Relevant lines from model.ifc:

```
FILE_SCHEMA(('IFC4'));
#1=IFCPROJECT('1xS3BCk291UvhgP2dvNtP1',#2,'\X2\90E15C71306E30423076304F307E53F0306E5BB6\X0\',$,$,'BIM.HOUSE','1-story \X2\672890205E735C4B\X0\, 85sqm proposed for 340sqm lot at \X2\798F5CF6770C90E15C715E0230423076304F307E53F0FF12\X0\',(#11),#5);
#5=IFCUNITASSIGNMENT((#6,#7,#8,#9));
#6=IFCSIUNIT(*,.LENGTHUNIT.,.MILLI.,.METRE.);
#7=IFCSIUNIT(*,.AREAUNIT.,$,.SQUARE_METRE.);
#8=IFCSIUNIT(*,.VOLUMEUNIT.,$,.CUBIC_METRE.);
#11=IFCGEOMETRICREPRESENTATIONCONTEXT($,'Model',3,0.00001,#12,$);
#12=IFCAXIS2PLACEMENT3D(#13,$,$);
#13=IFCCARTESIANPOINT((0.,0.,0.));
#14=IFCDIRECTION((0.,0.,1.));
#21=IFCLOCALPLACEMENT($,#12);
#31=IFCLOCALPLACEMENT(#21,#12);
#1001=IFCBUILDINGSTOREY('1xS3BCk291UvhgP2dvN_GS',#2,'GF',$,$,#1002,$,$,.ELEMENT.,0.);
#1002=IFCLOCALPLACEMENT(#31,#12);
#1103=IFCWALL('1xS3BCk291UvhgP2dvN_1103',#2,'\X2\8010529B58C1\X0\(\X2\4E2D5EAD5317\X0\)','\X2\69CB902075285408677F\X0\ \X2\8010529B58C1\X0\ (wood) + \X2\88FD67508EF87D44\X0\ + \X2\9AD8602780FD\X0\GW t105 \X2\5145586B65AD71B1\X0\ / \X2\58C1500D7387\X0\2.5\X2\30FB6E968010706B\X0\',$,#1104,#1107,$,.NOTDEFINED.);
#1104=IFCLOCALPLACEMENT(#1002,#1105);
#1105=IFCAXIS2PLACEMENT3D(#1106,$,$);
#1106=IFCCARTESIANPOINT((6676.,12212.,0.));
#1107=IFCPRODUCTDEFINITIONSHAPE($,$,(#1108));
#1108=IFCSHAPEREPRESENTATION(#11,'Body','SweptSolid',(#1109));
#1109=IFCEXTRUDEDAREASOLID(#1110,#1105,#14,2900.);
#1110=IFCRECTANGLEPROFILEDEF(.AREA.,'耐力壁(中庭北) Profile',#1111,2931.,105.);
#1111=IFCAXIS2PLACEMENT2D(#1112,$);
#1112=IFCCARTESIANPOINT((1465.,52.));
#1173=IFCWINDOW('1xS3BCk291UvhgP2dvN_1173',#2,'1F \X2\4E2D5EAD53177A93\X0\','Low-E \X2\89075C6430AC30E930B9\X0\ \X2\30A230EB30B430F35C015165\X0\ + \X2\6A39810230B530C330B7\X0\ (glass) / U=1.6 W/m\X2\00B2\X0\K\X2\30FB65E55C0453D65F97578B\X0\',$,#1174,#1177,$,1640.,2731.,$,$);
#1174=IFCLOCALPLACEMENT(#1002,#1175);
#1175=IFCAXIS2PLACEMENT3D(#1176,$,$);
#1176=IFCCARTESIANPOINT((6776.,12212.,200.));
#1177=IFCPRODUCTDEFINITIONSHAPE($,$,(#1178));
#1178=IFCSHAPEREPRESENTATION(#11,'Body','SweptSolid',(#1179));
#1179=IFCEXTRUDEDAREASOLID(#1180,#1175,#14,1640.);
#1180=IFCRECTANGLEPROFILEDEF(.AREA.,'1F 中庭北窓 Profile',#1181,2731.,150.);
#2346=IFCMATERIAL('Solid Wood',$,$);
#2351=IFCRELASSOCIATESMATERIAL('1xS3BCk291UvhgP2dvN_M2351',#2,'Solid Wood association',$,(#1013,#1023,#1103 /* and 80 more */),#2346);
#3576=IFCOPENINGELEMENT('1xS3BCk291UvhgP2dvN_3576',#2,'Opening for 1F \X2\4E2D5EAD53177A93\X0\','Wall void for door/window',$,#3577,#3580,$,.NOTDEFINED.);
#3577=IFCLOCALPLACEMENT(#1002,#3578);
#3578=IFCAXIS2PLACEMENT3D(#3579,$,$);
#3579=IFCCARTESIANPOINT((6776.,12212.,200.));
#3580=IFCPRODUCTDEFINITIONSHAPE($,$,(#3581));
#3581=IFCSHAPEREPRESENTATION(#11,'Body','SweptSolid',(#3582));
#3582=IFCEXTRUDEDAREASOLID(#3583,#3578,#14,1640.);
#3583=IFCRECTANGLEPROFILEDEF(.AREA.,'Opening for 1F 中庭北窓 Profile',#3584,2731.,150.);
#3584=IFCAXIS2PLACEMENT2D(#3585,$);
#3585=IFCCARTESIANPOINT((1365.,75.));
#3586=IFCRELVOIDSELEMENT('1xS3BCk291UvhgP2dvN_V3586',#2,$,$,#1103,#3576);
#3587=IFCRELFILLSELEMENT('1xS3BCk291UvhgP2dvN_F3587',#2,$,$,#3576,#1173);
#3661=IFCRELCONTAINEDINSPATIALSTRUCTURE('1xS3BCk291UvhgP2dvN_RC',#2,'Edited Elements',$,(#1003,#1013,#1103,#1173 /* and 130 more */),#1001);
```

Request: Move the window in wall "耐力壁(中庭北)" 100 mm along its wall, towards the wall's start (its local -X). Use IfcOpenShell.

```python
import ifcopenshell
import ifcopenshell.api.geometry
import ifcopenshell.util.placement
import ifcopenshell.util.unit

model = ifcopenshell.open("model.ifc")
unit_scale = ifcopenshell.util.unit.calculate_unit_scale(model)

window = model.by_id(1173)
opening = window.FillsVoids[0].RelatingOpeningElement
wall = opening.VoidsElements[0].RelatingBuildingElement

wall_matrix = ifcopenshell.util.placement.get_local_placement(wall.ObjectPlacement)
shift = wall_matrix[:3, 0] * -0.1 / unit_scale
before = ifcopenshell.util.placement.get_local_placement(window.ObjectPlacement)[:3, 3].copy()

# The window is not placed relative to its opening, so move both.
for product in (opening, window):
    matrix = ifcopenshell.util.placement.get_local_placement(product.ObjectPlacement)
    matrix[:3, 3] += shift
    ifcopenshell.api.geometry.edit_object_placement(model, product=product, matrix=matrix, is_si=False)

after = ifcopenshell.util.placement.get_local_placement(window.ObjectPlacement)[:3, 3]
print("window moved by", (after - before).round(3) + 0.0)

model.write("model-out.ifc")
```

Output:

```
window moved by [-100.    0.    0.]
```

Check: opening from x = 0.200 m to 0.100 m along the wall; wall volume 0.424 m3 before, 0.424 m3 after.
